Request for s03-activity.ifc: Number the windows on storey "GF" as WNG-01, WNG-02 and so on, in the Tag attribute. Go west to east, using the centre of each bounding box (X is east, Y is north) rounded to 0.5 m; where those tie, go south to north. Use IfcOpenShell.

First a look at what the model holds.

```python
import ifcopenshell
import ifcopenshell.util.element
import ifcopenshell.util.placement

model = ifcopenshell.open("s03-activity.ifc")
print(model.schema)
storey = next(s for s in model.by_type("IfcBuildingStorey") if s.Name == "GF")
windows = [e for e in ifcopenshell.util.element.get_decomposition(storey) if e.is_a("IfcWindow")]
for e in sorted(windows, key=lambda e: e.id()):
    origin = ifcopenshell.util.placement.get_local_placement(e.ObjectPlacement)[:3, 3]
    print(e.id(), e.Tag, e.Name, origin.round(2) + 0.0, sep=" | ")
```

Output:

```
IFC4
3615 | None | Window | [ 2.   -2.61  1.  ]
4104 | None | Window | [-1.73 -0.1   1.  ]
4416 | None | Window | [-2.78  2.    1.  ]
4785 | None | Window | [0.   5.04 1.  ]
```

```python
import ifcopenshell
import ifcopenshell.geom
import ifcopenshell.util.element
import ifcopenshell.util.shape

model = ifcopenshell.open("s03-activity.ifc")
settings = ifcopenshell.geom.settings()
settings.set("use-world-coords", True)


def centre(element):
    shape = ifcopenshell.geom.create_shape(settings, element)
    return ifcopenshell.util.shape.get_bbox_centroid(shape.geometry)


storey = next(s for s in model.by_type("IfcBuildingStorey") if s.Name == "GF")
windows = [e for e in ifcopenshell.util.element.get_decomposition(storey) if e.is_a("IfcWindow")]

# Insertion points can sit at a corner or the storey origin, so sort by the geometry (in metres).
centres = {e: centre(e) for e in windows}
windows.sort(key=lambda e: (round(centres[e][0] / 0.5), centres[e][1]))

for i, e in enumerate(windows, start=1):
    number = f"WNG-{i:02d}"
    e.Tag = number
    print(e.id(), number)

model.write("s03-activity_v2.ifc")
```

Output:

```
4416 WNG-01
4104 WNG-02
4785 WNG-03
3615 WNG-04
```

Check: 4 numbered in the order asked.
